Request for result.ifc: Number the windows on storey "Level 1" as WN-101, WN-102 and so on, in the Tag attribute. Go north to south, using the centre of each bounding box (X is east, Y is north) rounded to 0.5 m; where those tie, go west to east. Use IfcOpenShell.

First a look at what the model holds.

```python
import ifcopenshell
import ifcopenshell.util.element
import ifcopenshell.util.placement

model = ifcopenshell.open("result.ifc")
print(model.schema)
storey = next(s for s in model.by_type("IfcBuildingStorey") if s.Name == "Level 1")
windows = [e for e in ifcopenshell.util.element.get_decomposition(storey) if e.is_a("IfcWindow")]
for e in sorted(windows, key=lambda e: e.id()):
    origin = ifcopenshell.util.placement.get_local_placement(e.ObjectPlacement)[:3, 3]
    print(e.id(), e.Tag, e.Name, origin.round(2) + 0.0, sep=" | ")
```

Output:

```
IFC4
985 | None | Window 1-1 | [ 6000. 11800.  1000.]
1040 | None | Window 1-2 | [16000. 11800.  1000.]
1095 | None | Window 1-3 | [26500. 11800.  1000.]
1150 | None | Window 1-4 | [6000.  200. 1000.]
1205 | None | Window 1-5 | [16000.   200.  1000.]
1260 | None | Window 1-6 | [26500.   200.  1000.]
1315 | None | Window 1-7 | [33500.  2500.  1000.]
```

```python
import ifcopenshell
import ifcopenshell.geom
import ifcopenshell.util.element
import ifcopenshell.util.shape

model = ifcopenshell.open("result.ifc")
settings = ifcopenshell.geom.settings()
settings.set("use-world-coords", True)


def centre(element):
    shape = ifcopenshell.geom.create_shape(settings, element)
    return ifcopenshell.util.shape.get_bbox_centroid(shape.geometry)


storey = next(s for s in model.by_type("IfcBuildingStorey") if s.Name == "Level 1")
windows = [e for e in ifcopenshell.util.element.get_decomposition(storey) if e.is_a("IfcWindow")]

# Insertion points can sit at a corner or the storey origin, so sort by the geometry (in metres).
centres = {e: centre(e) for e in windows}
windows.sort(key=lambda e: (-round(centres[e][1] / 0.5), centres[e][0]))

for i, e in enumerate(windows, start=1):
    number = f"WN-1{i:02d}"
    e.Tag = number
    print(e.id(), number)

model.write("result_v2.ifc")
```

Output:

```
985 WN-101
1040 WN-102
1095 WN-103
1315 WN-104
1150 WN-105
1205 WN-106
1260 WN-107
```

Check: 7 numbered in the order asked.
